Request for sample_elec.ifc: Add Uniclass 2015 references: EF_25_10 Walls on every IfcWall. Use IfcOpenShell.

First a look at what the model holds.

```python
import ifcopenshell

model = ifcopenshell.open("sample_elec.ifc")
print(model.schema)
print("classifications:", [c.Name for c in model.by_type("IfcClassification")])
for ifc_class in ("IfcDoor", "IfcRoof", "IfcStair", "IfcWall", "IfcWindow"):
    print(ifc_class, len(model.by_type(ifc_class)))
```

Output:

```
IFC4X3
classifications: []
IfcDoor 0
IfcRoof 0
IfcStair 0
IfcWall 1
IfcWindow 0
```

```python
import ifcopenshell
import ifcopenshell.api.classification

model = ifcopenshell.open("sample_elec.ifc")

system = ifcopenshell.api.classification.add_classification(model, classification="Uniclass 2015")

codes = {
    "IfcWall": ("EF_25_10", "Walls"),
}
for ifc_class, (code, name) in codes.items():
    products = model.by_type(ifc_class)
    ifcopenshell.api.classification.add_reference(
        model, products=products, classification=system, identification=code, name=name
    )
    print(code, len(products))

model.write("sample_elec_edited.ifc")
```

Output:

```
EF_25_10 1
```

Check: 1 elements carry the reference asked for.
